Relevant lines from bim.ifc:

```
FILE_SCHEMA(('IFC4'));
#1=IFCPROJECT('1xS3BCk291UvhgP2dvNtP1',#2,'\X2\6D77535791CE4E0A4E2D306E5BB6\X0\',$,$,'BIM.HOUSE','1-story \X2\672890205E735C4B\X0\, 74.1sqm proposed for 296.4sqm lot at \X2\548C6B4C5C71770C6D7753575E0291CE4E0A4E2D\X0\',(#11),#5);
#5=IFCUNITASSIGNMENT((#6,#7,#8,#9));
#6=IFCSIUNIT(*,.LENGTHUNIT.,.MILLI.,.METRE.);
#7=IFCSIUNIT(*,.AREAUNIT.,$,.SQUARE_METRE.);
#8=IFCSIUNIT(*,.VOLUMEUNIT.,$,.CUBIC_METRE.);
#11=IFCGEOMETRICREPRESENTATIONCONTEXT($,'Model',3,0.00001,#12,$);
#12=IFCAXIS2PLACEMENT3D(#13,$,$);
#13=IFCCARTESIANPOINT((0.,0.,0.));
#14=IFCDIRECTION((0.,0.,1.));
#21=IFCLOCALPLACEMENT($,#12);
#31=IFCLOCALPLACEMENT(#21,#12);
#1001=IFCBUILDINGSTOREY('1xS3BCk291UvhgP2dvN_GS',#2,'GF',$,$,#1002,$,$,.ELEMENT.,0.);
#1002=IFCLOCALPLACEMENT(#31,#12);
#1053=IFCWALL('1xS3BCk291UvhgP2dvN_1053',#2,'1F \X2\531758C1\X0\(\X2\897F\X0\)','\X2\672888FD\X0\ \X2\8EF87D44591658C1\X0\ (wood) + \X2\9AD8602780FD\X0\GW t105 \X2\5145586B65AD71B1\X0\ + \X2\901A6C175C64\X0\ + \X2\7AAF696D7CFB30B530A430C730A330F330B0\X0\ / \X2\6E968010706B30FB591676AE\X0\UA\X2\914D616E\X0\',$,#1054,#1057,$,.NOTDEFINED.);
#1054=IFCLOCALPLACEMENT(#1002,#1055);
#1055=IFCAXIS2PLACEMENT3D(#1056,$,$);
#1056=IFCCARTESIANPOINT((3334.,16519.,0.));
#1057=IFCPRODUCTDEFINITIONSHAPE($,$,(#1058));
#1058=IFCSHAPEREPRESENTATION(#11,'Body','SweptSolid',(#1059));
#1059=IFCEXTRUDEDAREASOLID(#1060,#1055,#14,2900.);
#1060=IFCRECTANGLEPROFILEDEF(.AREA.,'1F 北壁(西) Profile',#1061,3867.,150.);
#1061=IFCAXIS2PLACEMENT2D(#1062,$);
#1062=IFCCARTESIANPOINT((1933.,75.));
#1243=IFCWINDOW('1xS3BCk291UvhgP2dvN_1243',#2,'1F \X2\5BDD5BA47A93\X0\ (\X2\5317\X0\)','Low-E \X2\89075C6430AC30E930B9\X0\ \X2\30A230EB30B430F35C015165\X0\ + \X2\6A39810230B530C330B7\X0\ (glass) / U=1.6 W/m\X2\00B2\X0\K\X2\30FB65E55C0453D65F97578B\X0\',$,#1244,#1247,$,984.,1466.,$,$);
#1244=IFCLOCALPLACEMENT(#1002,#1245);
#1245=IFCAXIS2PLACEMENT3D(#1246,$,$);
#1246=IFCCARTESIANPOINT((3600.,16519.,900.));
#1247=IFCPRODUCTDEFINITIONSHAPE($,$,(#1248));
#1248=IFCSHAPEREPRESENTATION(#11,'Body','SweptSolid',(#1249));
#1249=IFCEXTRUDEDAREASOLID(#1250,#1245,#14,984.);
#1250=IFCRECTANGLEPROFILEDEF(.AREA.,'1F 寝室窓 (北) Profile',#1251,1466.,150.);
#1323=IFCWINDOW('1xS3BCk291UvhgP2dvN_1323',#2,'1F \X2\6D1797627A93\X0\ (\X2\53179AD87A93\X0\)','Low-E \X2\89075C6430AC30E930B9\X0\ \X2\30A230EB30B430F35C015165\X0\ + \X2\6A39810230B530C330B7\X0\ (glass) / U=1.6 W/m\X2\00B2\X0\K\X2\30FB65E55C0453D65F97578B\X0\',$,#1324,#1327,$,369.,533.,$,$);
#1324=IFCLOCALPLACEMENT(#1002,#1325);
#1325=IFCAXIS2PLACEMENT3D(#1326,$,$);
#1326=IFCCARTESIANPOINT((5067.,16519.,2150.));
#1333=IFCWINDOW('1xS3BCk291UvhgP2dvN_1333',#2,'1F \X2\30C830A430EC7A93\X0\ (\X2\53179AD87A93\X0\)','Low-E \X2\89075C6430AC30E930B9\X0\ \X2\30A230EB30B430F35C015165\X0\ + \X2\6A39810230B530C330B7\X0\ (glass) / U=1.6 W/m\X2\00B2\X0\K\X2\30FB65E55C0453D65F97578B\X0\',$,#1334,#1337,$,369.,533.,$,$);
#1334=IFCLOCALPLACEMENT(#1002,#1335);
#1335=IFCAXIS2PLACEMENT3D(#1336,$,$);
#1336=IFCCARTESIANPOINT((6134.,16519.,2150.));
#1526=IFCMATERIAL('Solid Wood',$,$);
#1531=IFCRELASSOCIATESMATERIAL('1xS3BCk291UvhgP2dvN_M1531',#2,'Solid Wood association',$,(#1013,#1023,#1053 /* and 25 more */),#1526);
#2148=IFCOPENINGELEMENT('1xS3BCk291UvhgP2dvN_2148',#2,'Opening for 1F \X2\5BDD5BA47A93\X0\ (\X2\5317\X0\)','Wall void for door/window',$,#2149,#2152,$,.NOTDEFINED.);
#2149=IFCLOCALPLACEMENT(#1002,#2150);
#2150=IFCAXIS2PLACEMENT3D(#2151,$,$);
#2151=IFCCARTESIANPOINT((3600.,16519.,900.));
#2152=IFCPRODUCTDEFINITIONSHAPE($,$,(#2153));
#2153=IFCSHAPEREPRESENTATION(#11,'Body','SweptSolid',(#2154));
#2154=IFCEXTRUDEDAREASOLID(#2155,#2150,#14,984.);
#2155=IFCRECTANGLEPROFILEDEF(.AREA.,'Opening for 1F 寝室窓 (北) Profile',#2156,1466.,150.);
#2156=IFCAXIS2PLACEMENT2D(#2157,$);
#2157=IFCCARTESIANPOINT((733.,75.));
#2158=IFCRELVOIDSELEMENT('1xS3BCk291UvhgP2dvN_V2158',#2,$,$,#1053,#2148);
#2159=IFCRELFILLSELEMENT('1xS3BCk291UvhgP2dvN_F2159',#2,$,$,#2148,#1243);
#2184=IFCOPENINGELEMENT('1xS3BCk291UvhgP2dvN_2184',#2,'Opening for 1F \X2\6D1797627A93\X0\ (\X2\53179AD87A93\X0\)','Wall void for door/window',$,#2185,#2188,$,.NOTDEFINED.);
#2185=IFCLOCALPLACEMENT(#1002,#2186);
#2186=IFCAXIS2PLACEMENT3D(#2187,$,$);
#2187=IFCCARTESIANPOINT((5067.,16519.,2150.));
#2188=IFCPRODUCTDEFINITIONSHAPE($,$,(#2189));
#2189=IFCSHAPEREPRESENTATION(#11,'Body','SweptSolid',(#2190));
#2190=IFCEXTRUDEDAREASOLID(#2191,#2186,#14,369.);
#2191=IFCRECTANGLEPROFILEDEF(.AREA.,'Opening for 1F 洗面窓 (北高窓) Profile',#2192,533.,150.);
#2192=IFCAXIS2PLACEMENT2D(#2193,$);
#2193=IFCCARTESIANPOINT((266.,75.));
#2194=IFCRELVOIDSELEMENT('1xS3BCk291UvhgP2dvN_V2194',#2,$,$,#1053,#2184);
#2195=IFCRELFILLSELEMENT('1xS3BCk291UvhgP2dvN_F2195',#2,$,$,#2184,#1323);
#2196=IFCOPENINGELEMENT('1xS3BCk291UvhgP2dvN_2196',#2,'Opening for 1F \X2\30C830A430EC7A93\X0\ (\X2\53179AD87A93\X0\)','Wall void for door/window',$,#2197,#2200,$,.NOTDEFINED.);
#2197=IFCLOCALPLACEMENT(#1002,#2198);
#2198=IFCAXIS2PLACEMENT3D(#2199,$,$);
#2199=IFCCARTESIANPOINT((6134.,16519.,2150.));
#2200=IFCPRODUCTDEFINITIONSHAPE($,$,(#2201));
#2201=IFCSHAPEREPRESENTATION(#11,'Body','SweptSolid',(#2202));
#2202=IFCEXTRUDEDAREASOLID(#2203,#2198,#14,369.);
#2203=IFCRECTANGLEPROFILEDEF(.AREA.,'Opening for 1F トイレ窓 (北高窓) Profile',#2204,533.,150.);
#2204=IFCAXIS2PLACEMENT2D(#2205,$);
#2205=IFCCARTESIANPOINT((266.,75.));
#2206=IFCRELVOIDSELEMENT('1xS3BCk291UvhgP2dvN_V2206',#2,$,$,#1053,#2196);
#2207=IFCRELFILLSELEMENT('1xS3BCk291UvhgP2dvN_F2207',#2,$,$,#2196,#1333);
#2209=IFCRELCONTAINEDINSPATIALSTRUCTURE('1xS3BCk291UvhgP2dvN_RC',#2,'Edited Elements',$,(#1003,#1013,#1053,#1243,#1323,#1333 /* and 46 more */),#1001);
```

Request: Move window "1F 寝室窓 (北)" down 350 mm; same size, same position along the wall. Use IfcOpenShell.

```python
import numpy as np
import ifcopenshell
import ifcopenshell.api.geometry
import ifcopenshell.util.placement
import ifcopenshell.util.unit

model = ifcopenshell.open("bim.ifc")
unit_scale = ifcopenshell.util.unit.calculate_unit_scale(model)

window = model.by_guid("1xS3BCk291UvhgP2dvN_1243")
opening = window.FillsVoids[0].RelatingOpeningElement
dz = -0.35 / unit_scale

shift = np.array([0.0, 0.0, dz])
# The window is not placed relative to its opening, so move both.
for product in (opening, window):
    matrix = ifcopenshell.util.placement.get_local_placement(product.ObjectPlacement)
    matrix[:3, 3] += shift
    ifcopenshell.api.geometry.edit_object_placement(model, product=product, matrix=matrix, is_si=False)

print(f"moved by {dz * unit_scale:+.3f} m")

model.write("bim_v2.ifc")
```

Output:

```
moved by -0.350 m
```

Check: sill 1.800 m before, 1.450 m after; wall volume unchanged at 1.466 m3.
